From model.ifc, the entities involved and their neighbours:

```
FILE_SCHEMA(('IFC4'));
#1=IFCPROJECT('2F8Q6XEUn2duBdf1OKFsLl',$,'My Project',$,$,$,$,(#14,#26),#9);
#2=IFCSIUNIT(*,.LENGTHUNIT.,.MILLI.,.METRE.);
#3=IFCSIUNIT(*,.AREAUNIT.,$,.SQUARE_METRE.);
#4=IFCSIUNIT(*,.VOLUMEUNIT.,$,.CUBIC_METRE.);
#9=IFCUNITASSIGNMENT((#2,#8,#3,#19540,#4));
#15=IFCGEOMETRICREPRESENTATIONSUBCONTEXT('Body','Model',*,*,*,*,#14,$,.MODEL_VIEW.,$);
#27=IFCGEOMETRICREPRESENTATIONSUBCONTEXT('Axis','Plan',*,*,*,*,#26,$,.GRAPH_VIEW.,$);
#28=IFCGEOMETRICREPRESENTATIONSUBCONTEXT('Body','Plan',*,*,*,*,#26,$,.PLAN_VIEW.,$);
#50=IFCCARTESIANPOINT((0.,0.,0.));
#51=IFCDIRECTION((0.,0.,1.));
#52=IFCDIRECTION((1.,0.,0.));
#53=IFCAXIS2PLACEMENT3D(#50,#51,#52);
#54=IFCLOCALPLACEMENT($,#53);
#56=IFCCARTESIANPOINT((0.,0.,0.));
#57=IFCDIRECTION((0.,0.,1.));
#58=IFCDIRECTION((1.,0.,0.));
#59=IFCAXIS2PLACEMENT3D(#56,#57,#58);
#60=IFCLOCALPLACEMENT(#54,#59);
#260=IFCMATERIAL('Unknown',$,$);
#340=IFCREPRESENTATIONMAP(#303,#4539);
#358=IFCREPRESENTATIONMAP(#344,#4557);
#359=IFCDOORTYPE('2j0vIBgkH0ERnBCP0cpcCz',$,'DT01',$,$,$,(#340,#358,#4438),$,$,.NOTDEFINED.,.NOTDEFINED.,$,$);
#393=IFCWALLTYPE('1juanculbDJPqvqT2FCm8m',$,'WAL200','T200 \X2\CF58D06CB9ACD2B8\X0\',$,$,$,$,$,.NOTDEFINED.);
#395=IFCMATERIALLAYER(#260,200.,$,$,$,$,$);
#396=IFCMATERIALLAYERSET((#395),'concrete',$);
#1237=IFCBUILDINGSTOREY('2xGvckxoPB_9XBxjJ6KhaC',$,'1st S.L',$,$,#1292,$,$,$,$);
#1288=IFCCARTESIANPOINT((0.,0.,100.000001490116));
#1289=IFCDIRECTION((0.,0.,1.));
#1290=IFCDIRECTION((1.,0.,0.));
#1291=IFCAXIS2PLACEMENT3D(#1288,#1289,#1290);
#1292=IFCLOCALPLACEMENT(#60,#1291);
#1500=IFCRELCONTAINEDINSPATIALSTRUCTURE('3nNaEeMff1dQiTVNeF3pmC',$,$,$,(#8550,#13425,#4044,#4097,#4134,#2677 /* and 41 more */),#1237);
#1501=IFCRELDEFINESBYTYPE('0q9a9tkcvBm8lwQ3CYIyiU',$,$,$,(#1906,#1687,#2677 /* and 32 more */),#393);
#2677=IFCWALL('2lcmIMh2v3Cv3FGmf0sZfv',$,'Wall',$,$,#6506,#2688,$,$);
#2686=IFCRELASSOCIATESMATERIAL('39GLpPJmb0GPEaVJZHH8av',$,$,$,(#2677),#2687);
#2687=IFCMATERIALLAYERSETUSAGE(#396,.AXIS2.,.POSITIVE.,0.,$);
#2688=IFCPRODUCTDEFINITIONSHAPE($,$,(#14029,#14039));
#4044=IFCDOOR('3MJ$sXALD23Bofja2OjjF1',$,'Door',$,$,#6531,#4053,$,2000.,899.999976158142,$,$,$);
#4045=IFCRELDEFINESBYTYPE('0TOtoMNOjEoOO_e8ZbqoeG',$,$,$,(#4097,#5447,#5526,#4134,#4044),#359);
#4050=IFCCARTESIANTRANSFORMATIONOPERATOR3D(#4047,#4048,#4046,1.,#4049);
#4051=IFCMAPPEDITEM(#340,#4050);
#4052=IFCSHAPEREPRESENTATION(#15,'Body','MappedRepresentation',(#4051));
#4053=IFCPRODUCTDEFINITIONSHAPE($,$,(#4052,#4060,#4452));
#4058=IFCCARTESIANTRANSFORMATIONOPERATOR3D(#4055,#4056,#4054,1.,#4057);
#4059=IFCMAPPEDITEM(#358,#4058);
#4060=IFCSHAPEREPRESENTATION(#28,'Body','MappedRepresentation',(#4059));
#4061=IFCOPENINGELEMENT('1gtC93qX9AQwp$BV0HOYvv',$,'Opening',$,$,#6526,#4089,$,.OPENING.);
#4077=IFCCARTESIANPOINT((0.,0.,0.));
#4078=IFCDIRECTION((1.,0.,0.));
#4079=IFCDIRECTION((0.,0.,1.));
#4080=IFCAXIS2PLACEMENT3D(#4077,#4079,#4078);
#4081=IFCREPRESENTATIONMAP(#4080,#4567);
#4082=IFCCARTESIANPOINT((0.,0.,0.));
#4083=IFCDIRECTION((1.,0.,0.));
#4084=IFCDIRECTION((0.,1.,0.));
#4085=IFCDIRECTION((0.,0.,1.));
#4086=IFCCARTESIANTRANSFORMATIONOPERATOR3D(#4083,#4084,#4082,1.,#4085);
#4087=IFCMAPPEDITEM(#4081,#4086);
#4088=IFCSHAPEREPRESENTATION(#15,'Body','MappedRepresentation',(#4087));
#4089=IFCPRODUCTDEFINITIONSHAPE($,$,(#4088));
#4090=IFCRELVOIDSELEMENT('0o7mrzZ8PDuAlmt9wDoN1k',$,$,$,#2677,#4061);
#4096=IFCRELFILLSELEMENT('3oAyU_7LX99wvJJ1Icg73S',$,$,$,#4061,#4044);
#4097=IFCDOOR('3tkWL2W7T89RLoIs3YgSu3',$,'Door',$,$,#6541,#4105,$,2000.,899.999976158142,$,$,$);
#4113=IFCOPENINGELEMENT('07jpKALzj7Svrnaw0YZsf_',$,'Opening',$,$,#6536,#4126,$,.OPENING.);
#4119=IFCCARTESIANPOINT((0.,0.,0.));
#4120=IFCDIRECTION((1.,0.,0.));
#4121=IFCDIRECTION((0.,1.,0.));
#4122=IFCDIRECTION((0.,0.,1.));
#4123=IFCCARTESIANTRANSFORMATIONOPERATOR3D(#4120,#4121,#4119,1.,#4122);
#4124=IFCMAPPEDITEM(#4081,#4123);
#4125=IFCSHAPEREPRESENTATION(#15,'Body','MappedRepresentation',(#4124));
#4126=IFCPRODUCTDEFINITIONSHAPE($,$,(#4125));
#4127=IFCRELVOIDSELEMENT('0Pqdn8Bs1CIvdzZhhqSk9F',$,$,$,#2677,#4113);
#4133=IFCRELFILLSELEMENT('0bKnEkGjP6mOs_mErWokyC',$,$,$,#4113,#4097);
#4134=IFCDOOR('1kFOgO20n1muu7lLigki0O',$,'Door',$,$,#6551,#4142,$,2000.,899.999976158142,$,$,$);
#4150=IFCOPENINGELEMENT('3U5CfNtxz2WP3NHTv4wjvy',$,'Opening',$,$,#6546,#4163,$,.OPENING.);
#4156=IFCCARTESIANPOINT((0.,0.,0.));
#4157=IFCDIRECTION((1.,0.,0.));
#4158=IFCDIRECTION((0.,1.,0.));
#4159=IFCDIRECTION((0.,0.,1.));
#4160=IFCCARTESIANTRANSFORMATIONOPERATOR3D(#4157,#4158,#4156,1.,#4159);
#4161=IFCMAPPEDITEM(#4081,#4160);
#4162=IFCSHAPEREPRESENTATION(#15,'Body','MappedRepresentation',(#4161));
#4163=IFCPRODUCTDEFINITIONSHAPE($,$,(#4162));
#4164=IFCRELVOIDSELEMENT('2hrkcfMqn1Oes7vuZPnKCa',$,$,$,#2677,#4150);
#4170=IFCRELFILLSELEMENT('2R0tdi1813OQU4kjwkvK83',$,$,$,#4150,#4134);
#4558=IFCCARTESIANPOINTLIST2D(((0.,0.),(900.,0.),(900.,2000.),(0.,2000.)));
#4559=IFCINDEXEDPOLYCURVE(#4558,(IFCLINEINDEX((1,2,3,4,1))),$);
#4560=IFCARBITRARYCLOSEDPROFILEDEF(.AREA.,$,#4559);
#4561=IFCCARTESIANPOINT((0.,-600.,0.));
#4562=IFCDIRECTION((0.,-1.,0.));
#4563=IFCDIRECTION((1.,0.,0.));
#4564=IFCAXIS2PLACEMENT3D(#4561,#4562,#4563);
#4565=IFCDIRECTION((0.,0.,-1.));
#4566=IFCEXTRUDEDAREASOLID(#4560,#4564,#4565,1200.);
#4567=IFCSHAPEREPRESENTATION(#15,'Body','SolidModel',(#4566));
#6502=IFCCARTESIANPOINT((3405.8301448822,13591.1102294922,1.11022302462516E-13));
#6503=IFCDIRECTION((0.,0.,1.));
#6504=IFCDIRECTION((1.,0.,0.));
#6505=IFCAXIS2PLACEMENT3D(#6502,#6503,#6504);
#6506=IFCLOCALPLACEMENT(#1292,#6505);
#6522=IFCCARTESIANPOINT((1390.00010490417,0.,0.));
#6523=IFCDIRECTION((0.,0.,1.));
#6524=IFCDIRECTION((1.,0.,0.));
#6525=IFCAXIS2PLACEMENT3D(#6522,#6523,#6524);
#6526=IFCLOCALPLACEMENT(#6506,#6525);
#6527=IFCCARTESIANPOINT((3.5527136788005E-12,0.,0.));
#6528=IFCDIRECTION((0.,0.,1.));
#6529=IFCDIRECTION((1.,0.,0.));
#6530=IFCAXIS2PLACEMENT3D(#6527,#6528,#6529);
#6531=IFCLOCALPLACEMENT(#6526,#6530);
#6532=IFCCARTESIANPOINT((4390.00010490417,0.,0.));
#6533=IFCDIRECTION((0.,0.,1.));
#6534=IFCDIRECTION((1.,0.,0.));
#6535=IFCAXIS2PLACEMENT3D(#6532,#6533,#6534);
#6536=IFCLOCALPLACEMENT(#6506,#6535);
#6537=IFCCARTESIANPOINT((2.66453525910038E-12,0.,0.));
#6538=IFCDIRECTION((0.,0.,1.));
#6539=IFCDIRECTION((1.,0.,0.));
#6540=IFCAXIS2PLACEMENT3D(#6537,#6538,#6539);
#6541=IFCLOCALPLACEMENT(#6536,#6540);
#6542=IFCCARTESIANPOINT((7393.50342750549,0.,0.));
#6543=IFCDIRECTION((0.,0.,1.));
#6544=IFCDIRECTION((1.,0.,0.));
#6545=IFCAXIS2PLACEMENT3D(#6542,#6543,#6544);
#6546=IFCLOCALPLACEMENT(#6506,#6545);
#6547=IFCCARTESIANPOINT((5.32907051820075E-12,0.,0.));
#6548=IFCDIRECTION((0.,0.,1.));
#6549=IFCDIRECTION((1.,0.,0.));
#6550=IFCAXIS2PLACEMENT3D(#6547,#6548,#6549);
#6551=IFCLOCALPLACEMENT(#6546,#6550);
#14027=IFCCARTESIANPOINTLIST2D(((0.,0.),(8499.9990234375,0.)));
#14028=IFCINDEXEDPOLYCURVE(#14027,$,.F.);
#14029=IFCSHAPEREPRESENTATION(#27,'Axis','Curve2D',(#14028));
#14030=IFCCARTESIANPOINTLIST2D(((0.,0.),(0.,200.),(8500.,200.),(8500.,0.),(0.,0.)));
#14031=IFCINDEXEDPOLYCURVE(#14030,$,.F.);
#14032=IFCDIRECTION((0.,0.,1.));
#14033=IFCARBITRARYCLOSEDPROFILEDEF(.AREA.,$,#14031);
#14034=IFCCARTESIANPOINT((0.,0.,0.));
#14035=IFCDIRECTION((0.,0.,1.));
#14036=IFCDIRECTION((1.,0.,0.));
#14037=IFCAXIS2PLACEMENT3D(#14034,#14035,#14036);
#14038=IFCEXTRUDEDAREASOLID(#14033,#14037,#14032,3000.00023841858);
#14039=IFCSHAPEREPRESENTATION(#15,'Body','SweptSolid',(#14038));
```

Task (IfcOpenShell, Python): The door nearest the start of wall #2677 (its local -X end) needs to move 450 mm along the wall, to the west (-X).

```python
import ifcopenshell
import ifcopenshell.api.geometry
import ifcopenshell.util.placement
import ifcopenshell.util.unit

model = ifcopenshell.open("model.ifc")
unit_scale = ifcopenshell.util.unit.calculate_unit_scale(model)

door = model.by_guid("3MJ$sXALD23Bofja2OjjF1")
opening = door.FillsVoids[0].RelatingOpeningElement
wall = opening.VoidsElements[0].RelatingBuildingElement

wall_matrix = ifcopenshell.util.placement.get_local_placement(wall.ObjectPlacement)
shift = wall_matrix[:3, 0] * -0.45 / unit_scale
before = ifcopenshell.util.placement.get_local_placement(door.ObjectPlacement)[:3, 3].copy()

# The door is placed relative to its opening, so it follows when the opening moves.
matrix = ifcopenshell.util.placement.get_local_placement(opening.ObjectPlacement)
matrix[:3, 3] += shift
ifcopenshell.api.geometry.edit_object_placement(
    model, product=opening, matrix=matrix, is_si=False, should_transform_children=True
)

after = ifcopenshell.util.placement.get_local_placement(door.ObjectPlacement)[:3, 3]
print("door moved by", (after - before).round(3) + 0.0)

model.write("model_edited.ifc")
```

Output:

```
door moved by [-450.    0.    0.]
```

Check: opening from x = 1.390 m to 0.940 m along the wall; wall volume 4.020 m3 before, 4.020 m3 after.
